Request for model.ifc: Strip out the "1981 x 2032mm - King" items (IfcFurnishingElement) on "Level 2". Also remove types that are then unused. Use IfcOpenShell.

First a look at what the model holds.

```python
import ifcopenshell
import ifcopenshell.util.element

model = ifcopenshell.open("model.ifc")
print(model.schema)
storey = next(s for s in model.by_type("IfcBuildingStorey") if s.Name == "Level 2")
furniture = [e for e in ifcopenshell.util.element.get_decomposition(storey) if e.is_a("IfcFurnishingElement")]
seen = {}
for e in furniture:
    element_type = ifcopenshell.util.element.get_type(e)
    name = element_type.Name if element_type not in (None, e) else None
    seen[name] = seen.get(name, 0) + 1
for name, count in sorted(seen.items(), key=str):
    print(count, "x", name)
```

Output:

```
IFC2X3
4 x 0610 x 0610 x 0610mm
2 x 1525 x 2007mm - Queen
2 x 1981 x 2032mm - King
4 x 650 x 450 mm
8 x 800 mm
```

```python
import ifcopenshell
import ifcopenshell.api.root
import ifcopenshell.util.element

model = ifcopenshell.open("model.ifc")

storey = next(s for s in model.by_type("IfcBuildingStorey") if s.Name == "Level 2")
furniture = [e for e in ifcopenshell.util.element.get_decomposition(storey) if e.is_a("IfcFurnishingElement")]
targets = [e for e in furniture if (t := ifcopenshell.util.element.get_type(e)) not in (None, e) and t.Name == "1981 x 2032mm - King"]
types = {ifcopenshell.util.element.get_type(e) for e in targets} - {None, *targets}

for e in targets:
    ifcopenshell.api.root.remove_product(model, product=e)
print(len(targets), "removed")

unused = [t for t in types if not ifcopenshell.util.element.get_types(t)]
for t in unused:
    ifcopenshell.api.root.remove_product(model, product=t)
print(len(unused), "unused types removed")

model.write("model_v2.ifc")
```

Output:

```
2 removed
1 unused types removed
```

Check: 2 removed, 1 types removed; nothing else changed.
